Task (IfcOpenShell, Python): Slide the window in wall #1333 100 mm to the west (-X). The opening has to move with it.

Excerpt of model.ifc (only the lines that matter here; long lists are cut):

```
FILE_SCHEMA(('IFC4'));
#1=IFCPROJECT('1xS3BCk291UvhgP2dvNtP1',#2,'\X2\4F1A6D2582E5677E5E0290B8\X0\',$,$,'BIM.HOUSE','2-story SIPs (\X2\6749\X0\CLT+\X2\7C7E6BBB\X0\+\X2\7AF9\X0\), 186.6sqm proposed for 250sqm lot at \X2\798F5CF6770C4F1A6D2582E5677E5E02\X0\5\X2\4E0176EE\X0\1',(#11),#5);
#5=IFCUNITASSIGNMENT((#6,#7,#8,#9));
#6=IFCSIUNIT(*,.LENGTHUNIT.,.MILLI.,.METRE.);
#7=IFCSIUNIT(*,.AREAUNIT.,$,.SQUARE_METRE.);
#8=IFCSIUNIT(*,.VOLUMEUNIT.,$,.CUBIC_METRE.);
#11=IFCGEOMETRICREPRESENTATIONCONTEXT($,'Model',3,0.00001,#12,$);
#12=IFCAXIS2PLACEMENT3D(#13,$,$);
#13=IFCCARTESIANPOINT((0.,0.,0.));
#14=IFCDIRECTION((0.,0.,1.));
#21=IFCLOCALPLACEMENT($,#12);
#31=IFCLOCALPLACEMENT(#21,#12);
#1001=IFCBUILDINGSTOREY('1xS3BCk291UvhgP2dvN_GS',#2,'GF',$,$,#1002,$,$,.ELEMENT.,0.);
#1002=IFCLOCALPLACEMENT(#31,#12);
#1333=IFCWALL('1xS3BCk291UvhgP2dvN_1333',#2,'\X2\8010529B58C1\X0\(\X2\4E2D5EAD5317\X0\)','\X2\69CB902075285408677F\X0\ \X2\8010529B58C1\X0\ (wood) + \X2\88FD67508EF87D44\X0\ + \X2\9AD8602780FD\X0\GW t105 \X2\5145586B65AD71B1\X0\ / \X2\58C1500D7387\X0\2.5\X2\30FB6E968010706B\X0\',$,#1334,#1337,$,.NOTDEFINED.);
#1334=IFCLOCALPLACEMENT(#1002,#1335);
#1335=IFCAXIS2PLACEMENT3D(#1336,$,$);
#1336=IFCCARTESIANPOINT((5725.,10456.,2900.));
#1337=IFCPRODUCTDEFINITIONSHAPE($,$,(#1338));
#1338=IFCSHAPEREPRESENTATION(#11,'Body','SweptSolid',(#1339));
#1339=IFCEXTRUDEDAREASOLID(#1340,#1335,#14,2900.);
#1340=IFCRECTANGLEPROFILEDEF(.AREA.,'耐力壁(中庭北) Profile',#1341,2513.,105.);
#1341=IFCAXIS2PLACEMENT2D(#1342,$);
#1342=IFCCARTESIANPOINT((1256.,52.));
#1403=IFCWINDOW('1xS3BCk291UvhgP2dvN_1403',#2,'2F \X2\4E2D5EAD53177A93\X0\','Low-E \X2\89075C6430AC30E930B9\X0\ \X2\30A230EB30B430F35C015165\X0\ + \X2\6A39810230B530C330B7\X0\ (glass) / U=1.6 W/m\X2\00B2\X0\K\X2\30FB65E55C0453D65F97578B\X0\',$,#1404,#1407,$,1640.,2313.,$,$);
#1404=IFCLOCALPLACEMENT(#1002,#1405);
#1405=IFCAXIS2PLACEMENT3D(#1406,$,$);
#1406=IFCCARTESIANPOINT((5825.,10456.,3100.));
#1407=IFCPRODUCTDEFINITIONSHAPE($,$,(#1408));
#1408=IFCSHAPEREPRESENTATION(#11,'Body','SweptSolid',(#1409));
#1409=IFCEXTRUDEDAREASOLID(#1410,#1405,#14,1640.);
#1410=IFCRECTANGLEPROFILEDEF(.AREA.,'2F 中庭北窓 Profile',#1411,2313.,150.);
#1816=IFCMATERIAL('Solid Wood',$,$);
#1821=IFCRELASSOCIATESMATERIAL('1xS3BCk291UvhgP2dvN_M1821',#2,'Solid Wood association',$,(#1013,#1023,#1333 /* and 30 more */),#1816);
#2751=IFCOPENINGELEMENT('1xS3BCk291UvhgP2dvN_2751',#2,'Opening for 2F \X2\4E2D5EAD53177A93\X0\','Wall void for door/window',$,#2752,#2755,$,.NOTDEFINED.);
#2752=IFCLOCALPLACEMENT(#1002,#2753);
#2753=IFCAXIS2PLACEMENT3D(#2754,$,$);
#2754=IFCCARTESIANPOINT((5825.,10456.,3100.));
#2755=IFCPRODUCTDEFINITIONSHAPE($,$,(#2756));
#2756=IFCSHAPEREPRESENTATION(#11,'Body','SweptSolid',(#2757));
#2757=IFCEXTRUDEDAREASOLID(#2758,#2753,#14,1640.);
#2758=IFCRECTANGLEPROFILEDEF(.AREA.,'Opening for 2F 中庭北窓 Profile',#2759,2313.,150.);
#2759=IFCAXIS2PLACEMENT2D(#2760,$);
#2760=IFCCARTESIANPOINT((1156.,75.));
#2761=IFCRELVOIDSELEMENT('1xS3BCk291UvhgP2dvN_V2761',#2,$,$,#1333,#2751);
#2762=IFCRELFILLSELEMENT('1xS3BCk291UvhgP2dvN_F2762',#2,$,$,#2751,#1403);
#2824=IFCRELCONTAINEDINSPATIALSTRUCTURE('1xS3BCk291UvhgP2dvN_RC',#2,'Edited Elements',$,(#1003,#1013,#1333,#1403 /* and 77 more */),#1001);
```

```python
import ifcopenshell
import ifcopenshell.api.geometry
import ifcopenshell.util.placement

model = ifcopenshell.open("model.ifc")

window = model.by_guid("1xS3BCk291UvhgP2dvN_1403")
opening = window.FillsVoids[0].RelatingOpeningElement
wall = opening.VoidsElements[0].RelatingBuildingElement

wall_matrix = ifcopenshell.util.placement.get_local_placement(wall.ObjectPlacement)
shift = wall_matrix[:3, 0] * -100.0
before = ifcopenshell.util.placement.get_local_placement(window.ObjectPlacement)[:3, 3].copy()

# The window is not placed relative to its opening, so move both.
for product in (opening, window):
    matrix = ifcopenshell.util.placement.get_local_placement(product.ObjectPlacement)
    matrix[:3, 3] += shift
    ifcopenshell.api.geometry.edit_object_placement(model, product=product, matrix=matrix, is_si=False)

after = ifcopenshell.util.placement.get_local_placement(window.ObjectPlacement)[:3, 3]
print("window moved by", (after - before).round(3) + 0.0)

model.write("model_updated.ifc")
```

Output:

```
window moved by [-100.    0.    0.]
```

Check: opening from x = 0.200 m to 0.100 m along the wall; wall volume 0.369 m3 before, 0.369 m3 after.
